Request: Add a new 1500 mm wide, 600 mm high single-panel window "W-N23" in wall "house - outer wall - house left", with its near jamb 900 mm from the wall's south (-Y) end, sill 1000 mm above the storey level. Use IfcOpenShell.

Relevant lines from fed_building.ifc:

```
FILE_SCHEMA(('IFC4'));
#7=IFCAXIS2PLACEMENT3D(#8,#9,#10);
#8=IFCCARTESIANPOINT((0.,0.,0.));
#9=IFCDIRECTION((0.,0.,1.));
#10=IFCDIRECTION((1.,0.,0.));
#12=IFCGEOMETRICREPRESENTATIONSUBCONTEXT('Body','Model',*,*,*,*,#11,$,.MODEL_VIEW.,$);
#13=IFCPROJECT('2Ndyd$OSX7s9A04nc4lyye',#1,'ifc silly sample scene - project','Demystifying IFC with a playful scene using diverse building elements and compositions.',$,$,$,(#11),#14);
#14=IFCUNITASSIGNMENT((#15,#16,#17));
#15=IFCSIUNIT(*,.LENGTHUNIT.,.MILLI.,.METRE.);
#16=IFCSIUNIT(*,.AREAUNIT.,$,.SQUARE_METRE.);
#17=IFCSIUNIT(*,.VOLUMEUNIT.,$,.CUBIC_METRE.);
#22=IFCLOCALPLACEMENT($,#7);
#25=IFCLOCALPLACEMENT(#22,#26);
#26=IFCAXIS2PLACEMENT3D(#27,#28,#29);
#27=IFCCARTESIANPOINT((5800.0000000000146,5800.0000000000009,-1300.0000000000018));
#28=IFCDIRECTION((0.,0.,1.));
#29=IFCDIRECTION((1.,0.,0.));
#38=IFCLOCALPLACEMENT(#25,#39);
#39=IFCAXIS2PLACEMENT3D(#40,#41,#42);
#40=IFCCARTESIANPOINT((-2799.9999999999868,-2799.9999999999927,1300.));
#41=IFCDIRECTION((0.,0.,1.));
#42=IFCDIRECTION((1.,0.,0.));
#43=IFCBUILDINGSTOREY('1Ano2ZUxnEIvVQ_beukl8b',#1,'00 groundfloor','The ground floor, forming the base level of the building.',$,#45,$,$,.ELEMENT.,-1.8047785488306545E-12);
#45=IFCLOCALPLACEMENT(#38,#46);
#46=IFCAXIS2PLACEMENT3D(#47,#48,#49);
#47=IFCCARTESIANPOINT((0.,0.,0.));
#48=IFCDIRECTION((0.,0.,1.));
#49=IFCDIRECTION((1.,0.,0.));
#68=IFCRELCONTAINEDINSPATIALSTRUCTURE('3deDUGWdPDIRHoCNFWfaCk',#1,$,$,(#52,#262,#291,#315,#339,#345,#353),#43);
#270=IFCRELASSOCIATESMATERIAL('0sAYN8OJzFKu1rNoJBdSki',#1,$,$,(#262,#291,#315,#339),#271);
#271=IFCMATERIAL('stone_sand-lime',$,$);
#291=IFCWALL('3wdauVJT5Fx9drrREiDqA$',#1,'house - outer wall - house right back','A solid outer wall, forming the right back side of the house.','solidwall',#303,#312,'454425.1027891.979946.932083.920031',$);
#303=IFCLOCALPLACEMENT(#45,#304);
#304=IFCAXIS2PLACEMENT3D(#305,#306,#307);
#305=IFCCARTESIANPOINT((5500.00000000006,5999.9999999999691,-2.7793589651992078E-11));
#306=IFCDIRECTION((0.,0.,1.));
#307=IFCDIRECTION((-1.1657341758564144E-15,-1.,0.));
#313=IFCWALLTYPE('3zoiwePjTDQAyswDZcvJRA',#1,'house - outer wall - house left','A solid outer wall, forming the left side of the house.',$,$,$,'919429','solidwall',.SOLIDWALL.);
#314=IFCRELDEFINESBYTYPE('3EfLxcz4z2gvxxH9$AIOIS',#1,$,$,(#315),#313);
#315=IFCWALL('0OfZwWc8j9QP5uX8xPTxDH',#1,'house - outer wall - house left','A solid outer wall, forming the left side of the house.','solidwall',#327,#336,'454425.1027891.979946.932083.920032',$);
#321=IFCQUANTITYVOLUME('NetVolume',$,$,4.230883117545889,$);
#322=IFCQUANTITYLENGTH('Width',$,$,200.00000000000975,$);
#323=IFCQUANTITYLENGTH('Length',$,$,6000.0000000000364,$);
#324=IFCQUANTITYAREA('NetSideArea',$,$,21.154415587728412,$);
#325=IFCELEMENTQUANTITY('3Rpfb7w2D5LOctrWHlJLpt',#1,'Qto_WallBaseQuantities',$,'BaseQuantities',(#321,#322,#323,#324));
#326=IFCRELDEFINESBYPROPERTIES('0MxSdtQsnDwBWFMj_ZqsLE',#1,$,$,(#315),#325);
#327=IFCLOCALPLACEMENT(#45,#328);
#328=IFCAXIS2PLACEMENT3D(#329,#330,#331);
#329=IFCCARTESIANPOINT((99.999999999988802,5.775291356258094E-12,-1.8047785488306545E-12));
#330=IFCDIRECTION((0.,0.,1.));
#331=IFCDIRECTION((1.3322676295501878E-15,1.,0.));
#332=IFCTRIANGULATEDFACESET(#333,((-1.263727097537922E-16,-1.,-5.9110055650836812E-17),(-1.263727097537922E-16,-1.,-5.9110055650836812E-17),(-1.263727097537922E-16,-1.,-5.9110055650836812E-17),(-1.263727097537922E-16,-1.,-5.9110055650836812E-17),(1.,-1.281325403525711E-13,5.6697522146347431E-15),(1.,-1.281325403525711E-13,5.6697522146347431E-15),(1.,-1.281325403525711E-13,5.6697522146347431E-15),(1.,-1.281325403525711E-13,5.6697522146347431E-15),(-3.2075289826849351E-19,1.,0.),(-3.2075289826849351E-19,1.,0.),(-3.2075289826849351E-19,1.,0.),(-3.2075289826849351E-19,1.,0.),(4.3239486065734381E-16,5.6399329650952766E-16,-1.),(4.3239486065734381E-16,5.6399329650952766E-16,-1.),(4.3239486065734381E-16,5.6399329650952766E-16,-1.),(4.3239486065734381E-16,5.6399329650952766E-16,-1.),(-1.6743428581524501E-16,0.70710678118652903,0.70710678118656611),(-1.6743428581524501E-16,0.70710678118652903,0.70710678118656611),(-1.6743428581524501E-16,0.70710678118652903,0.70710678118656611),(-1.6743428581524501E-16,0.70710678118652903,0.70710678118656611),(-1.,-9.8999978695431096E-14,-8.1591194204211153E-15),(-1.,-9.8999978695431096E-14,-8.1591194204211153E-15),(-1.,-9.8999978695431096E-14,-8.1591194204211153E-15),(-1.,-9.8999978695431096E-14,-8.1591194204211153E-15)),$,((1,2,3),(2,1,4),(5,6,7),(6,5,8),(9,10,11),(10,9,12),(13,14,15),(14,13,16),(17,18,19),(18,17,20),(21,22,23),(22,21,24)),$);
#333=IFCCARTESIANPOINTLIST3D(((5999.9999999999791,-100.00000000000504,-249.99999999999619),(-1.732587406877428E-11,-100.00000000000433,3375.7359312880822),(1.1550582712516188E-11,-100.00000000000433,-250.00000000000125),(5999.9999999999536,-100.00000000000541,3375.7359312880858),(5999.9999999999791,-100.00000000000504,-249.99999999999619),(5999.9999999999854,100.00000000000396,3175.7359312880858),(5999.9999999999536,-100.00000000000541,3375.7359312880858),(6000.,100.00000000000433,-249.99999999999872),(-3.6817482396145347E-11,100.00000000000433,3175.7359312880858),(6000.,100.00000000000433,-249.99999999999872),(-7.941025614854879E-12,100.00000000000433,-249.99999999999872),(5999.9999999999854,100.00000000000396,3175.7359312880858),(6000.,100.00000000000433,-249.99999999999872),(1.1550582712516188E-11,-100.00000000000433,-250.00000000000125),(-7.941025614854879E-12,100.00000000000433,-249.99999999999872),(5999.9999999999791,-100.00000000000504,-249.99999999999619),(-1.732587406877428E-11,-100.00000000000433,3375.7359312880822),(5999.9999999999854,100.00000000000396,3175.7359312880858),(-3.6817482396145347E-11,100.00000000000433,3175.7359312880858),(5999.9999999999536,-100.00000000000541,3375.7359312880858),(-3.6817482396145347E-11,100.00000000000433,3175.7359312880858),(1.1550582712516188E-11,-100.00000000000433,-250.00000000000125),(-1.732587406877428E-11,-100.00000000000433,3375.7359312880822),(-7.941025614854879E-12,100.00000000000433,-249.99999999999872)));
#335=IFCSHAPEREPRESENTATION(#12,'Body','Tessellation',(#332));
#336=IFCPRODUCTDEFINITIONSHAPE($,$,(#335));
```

```python
import numpy as np
import ifcopenshell
import ifcopenshell.api.feature
import ifcopenshell.api.geometry
import ifcopenshell.api.pset
import ifcopenshell.api.root
import ifcopenshell.api.spatial
import ifcopenshell.geom
import ifcopenshell.util.element
import ifcopenshell.util.placement
import ifcopenshell.util.representation
import ifcopenshell.util.shape
import ifcopenshell.util.unit

model = ifcopenshell.open("fed_building.ifc")
unit_scale = ifcopenshell.util.unit.calculate_unit_scale(model)
area_scale = ifcopenshell.util.unit.calculate_unit_scale(model, "AREAUNIT")
volume_scale = ifcopenshell.util.unit.calculate_unit_scale(model, "VOLUMEUNIT")
settings = ifcopenshell.geom.settings()


def volume(element):
    """Net volume in cubic metres, openings subtracted."""
    shape = ifcopenshell.geom.create_shape(settings, element)
    return ifcopenshell.util.shape.get_volume(shape.geometry)


wall = model.by_guid("0OfZwWc8j9QP5uX8xPTxDH")
storey = ifcopenshell.util.element.get_container(wall, ifc_class="IfcBuildingStorey")
context = ifcopenshell.util.representation.get_context(model, "Model", "Body", "MODEL_VIEW")
before = volume(wall)

width, height, from_end, sill = 1.5, 0.6, 0.9, 1  # metres

# The wall runs along its own X axis, and the end named is its -X end.
wall_shape = ifcopenshell.geom.create_shape(settings, wall)
x, y, z = ifcopenshell.util.shape.get_vertices(wall_shape.geometry).T
start = x.min() + from_end
face, thickness = float(y.min()), float(y.max() - y.min())
wall_matrix = ifcopenshell.util.placement.get_local_placement(wall.ObjectPlacement)
level = ifcopenshell.util.placement.get_local_placement(storey.ObjectPlacement)[2, 3]


def in_wall(x, y):
    """Placement at x, y metres in the wall's axes, at sill height."""
    matrix = wall_matrix.copy()
    matrix[:, 3] = wall_matrix @ np.array([x / unit_scale, y / unit_scale, 0.0, 1.0])
    matrix[2, 3] = level + sill / unit_scale
    return matrix


# Opening: a box that overshoots both wall faces by 50 mm.
opening = ifcopenshell.api.root.create_entity(model, ifc_class="IfcOpeningElement", predefined_type="OPENING")
box = ifcopenshell.api.geometry.add_wall_representation(
    model, context=context, length=width, height=height, thickness=thickness + 0.1
)
ifcopenshell.api.geometry.assign_representation(model, product=opening, representation=box)
ifcopenshell.api.geometry.edit_object_placement(model, product=opening, matrix=in_wall(start, face - 0.05), is_si=False)
ifcopenshell.api.feature.add_feature(model, feature=opening, element=wall)

window = ifcopenshell.api.root.create_entity(model, ifc_class="IfcWindow", name="W-N23", predefined_type="WINDOW")
window.OverallWidth, window.OverallHeight = width / unit_scale, height / unit_scale
window.PartitioningType = "SINGLE_PANEL"
body = ifcopenshell.api.geometry.add_window_representation(
    model,
    context=context,
    overall_width=window.OverallWidth,
    overall_height=window.OverallHeight,
    partition_type="SINGLE_PANEL",
)
ifcopenshell.api.geometry.assign_representation(model, product=window, representation=body)
ifcopenshell.api.spatial.assign_container(model, products=[window], relating_structure=storey)
ifcopenshell.api.feature.add_filling(model, opening=opening, element=window)

# Centre the window in the wall's thickness.
ifcopenshell.api.geometry.edit_object_placement(model, product=window, matrix=in_wall(start, face), is_si=False)
window_shape = ifcopenshell.geom.create_shape(settings, window)
depth = ifcopenshell.util.shape.get_vertices(window_shape.geometry)[:, 1]
offset = face + thickness / 2 - (depth.min() + depth.max()) / 2
ifcopenshell.api.geometry.edit_object_placement(model, product=window, matrix=in_wall(start, offset), is_si=False)

after = volume(wall)

# Update the wall's stored quantities.
qto = model.by_id(ifcopenshell.util.element.get_pset(wall, "Qto_WallBaseQuantities", should_inherit=False)["id"])
ifcopenshell.api.pset.edit_qto(model, qto=qto, properties={
    "NetVolume": after / volume_scale,
    "NetSideArea": after / thickness / area_scale,
})

print(f"wall volume {before:.3f} -> {after:.3f} m3")

model.write("fed_building_v2.ifc")
```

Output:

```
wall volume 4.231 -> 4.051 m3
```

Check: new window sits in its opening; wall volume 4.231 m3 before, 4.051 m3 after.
